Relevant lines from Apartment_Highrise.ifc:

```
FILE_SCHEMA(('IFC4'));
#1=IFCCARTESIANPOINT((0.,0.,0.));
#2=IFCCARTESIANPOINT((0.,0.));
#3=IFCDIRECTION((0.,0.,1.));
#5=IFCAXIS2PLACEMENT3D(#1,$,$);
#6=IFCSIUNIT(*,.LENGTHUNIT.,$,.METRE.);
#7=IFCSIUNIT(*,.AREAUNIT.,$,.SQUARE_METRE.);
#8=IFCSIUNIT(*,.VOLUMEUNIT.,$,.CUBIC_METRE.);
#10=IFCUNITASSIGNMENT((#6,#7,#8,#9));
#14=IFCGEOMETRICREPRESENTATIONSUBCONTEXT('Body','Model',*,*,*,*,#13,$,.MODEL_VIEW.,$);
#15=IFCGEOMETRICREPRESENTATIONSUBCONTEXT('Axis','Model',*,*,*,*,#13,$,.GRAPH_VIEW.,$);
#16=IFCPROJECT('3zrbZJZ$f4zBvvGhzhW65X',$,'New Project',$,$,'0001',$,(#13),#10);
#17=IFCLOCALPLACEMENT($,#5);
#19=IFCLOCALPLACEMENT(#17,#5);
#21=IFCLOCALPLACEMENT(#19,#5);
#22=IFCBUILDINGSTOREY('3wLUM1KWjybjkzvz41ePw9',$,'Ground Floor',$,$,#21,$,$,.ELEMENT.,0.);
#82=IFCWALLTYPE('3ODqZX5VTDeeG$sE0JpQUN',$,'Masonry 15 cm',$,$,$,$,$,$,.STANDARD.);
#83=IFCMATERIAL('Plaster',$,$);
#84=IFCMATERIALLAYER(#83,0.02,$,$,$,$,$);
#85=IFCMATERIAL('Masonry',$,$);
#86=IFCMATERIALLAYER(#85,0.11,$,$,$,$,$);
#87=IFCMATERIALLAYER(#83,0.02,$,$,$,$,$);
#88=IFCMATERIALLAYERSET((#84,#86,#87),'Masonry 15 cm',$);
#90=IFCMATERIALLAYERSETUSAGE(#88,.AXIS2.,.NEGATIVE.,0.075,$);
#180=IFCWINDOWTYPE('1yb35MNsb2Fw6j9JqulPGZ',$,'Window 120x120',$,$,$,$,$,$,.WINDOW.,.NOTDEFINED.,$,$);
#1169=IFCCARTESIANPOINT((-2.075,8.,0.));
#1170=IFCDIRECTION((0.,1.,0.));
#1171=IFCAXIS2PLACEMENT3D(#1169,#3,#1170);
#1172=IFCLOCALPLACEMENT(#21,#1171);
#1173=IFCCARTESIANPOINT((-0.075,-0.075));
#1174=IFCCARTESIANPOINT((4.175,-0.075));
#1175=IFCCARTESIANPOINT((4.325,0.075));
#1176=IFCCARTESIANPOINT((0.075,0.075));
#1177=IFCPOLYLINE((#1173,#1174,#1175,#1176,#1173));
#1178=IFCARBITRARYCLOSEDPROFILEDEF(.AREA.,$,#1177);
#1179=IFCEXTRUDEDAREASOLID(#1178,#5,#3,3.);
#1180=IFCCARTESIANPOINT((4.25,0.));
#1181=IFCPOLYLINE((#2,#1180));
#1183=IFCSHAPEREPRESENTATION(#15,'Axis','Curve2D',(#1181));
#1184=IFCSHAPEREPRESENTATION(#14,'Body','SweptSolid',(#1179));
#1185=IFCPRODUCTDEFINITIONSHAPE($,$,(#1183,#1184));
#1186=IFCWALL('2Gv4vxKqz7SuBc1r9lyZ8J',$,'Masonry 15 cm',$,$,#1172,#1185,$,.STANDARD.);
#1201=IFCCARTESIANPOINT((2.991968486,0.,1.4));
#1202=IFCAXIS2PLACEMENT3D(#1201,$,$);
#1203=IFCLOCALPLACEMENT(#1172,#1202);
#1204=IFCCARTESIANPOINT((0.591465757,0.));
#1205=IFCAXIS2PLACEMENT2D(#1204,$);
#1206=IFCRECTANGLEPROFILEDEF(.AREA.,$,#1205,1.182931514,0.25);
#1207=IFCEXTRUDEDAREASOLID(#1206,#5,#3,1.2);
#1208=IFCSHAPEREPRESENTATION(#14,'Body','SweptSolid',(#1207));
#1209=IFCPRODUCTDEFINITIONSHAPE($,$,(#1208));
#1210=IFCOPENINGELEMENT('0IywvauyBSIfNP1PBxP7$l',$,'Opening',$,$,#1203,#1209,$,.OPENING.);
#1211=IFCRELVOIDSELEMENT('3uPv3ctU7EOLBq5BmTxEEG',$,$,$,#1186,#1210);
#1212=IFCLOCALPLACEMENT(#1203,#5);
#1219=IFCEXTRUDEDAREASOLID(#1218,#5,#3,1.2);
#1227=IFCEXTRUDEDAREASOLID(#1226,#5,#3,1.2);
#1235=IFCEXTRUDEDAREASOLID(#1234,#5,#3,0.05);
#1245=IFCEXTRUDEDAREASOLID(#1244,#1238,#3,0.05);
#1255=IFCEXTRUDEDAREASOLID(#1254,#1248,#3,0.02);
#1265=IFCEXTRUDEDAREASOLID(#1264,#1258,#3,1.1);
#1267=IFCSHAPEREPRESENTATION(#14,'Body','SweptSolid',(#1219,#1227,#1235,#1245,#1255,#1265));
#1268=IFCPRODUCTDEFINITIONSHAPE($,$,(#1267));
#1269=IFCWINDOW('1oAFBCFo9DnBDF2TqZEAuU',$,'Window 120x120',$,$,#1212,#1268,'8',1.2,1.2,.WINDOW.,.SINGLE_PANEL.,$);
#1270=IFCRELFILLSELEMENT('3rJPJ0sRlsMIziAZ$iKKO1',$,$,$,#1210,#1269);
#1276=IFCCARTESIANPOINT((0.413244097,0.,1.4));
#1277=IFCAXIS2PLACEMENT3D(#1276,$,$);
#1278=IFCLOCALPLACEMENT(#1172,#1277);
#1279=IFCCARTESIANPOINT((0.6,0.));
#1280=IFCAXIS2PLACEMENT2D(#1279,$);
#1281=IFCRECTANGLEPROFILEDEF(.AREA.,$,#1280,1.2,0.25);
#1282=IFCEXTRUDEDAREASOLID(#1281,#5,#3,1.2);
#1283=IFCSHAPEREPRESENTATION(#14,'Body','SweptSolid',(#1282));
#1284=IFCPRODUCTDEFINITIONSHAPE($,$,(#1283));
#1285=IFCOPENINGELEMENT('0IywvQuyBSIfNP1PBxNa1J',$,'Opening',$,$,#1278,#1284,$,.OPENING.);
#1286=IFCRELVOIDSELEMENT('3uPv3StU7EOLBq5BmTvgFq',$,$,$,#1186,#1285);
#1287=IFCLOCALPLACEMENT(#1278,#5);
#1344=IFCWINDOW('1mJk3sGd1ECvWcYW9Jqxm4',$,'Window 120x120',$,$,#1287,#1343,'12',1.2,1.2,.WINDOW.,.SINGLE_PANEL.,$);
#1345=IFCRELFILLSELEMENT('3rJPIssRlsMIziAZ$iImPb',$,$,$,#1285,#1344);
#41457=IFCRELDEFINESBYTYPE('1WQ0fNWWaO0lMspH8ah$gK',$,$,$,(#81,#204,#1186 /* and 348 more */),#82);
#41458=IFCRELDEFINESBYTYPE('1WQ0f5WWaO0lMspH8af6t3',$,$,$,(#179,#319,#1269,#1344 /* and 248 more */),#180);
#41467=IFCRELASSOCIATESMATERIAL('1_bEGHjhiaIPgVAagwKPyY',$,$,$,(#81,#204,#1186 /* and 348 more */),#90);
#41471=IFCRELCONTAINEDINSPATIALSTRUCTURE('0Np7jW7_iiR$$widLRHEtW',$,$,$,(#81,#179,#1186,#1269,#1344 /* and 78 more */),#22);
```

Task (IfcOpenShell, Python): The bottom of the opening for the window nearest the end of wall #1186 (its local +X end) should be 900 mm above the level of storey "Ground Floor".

```python
import numpy as np
import ifcopenshell
import ifcopenshell.api.geometry
import ifcopenshell.geom
import ifcopenshell.util.element
import ifcopenshell.util.placement
import ifcopenshell.util.shape
import ifcopenshell.util.unit

model = ifcopenshell.open("Apartment_Highrise.ifc")
unit_scale = ifcopenshell.util.unit.calculate_unit_scale(model)

window = model.by_guid("1oAFBCFo9DnBDF2TqZEAuU")
opening = window.FillsVoids[0].RelatingOpeningElement
storey = ifcopenshell.util.element.get_container(window, ifc_class="IfcBuildingStorey")
level = ifcopenshell.util.placement.get_local_placement(storey.ObjectPlacement)[2, 3]

# The opening's origin need not be at the sill, so measure its lowest point.
shape = ifcopenshell.geom.create_shape(ifcopenshell.geom.settings(), opening)
bottom = ifcopenshell.util.shape.get_shape_bottom_elevation(shape, shape.geometry) / unit_scale
dz = level + 0.9 - bottom

shift = np.array([0.0, 0.0, dz])
# The window is placed relative to its opening, so it follows when the opening moves.
matrix = ifcopenshell.util.placement.get_local_placement(opening.ObjectPlacement)
matrix[:3, 3] += shift
ifcopenshell.api.geometry.edit_object_placement(
    model, product=opening, matrix=matrix, is_si=False, should_transform_children=True
)

print(f"moved by {dz * unit_scale:+.3f} m")

model.write("Apartment_Highrise_updated.ifc")
```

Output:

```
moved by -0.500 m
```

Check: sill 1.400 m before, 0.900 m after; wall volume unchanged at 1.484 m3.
